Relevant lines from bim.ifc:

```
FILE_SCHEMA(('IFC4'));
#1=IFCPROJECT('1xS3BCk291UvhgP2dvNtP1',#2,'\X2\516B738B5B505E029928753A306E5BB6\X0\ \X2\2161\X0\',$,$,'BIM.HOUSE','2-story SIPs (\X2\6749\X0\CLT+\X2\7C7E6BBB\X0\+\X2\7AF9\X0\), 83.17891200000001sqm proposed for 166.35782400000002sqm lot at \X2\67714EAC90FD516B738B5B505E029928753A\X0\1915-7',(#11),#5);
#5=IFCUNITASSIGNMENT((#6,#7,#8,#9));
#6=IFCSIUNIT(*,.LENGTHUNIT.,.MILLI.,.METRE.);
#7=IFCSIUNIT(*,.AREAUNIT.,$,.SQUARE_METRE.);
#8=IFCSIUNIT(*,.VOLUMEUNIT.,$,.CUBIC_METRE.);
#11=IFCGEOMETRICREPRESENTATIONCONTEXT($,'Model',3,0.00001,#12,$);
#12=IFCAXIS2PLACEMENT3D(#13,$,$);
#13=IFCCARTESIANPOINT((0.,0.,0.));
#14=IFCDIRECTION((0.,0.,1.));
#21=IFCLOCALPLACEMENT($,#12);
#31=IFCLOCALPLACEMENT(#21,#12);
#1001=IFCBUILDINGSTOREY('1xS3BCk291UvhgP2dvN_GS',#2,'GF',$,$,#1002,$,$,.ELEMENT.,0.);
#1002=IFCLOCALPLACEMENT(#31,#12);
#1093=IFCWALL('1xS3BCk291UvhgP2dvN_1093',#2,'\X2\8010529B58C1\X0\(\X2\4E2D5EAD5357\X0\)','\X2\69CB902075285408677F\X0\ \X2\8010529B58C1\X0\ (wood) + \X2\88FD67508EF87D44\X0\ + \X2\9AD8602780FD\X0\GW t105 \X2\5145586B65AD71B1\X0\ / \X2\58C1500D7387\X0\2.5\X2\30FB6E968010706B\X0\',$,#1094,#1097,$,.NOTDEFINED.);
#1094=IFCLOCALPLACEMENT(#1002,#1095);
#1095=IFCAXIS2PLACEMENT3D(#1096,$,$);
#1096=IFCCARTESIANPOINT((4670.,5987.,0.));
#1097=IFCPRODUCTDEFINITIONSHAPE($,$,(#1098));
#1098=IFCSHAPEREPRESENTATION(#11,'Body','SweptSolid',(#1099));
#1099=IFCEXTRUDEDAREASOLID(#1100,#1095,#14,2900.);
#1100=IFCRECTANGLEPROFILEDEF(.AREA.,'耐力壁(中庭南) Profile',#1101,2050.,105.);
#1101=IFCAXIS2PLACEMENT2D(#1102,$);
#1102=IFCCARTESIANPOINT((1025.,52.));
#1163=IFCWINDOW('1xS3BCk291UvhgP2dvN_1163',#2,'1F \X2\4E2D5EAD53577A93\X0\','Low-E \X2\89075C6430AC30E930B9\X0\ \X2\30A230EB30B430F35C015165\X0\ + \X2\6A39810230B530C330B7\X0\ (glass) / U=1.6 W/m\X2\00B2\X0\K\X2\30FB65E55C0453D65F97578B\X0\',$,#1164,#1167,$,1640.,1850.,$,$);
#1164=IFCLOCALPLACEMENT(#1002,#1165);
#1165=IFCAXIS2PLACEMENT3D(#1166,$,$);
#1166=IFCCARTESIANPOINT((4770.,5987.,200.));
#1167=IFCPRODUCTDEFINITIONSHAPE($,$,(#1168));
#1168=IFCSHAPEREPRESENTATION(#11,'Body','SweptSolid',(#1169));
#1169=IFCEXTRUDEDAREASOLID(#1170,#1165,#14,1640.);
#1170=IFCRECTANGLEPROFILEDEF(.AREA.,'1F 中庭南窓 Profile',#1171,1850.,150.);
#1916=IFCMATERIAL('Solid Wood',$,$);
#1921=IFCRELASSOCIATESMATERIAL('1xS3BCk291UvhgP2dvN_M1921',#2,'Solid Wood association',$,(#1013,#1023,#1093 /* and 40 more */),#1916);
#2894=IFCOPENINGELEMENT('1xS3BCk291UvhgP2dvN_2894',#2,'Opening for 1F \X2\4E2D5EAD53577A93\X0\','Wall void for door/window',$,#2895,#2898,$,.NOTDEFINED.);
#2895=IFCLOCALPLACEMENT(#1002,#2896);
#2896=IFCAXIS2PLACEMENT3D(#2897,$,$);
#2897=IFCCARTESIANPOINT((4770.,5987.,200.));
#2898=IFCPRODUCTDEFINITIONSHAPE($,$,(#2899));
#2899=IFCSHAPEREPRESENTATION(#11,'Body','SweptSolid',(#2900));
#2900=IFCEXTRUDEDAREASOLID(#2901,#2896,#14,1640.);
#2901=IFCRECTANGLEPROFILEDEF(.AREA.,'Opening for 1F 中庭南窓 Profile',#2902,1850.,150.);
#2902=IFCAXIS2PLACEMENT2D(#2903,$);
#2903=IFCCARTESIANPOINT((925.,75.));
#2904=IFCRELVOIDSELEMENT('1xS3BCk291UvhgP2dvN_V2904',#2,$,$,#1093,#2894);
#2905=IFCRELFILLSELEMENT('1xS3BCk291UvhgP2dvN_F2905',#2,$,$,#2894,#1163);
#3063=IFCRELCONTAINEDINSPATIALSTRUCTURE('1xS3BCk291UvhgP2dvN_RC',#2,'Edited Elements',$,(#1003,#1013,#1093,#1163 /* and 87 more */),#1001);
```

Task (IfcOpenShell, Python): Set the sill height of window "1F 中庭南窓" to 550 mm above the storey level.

```python
import numpy as np
import ifcopenshell
import ifcopenshell.api.geometry
import ifcopenshell.geom
import ifcopenshell.util.element
import ifcopenshell.util.placement
import ifcopenshell.util.shape
import ifcopenshell.util.unit

model = ifcopenshell.open("bim.ifc")
unit_scale = ifcopenshell.util.unit.calculate_unit_scale(model)

window = model.by_guid("1xS3BCk291UvhgP2dvN_1163")
opening = window.FillsVoids[0].RelatingOpeningElement
storey = ifcopenshell.util.element.get_container(window, ifc_class="IfcBuildingStorey")
level = ifcopenshell.util.placement.get_local_placement(storey.ObjectPlacement)[2, 3]

# The opening's origin need not be at the sill, so measure its lowest point.
shape = ifcopenshell.geom.create_shape(ifcopenshell.geom.settings(), opening)
bottom = ifcopenshell.util.shape.get_shape_bottom_elevation(shape, shape.geometry) / unit_scale
dz = level + 0.55 / unit_scale - bottom

shift = np.array([0.0, 0.0, dz])
# The window is not placed relative to its opening, so move both.
for product in (opening, window):
    matrix = ifcopenshell.util.placement.get_local_placement(product.ObjectPlacement)
    matrix[:3, 3] += shift
    ifcopenshell.api.geometry.edit_object_placement(model, product=product, matrix=matrix, is_si=False)

print(f"moved by {dz * unit_scale:+.3f} m")

model.write("bim_edited.ifc")
```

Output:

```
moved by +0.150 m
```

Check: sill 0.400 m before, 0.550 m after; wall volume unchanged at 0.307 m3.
